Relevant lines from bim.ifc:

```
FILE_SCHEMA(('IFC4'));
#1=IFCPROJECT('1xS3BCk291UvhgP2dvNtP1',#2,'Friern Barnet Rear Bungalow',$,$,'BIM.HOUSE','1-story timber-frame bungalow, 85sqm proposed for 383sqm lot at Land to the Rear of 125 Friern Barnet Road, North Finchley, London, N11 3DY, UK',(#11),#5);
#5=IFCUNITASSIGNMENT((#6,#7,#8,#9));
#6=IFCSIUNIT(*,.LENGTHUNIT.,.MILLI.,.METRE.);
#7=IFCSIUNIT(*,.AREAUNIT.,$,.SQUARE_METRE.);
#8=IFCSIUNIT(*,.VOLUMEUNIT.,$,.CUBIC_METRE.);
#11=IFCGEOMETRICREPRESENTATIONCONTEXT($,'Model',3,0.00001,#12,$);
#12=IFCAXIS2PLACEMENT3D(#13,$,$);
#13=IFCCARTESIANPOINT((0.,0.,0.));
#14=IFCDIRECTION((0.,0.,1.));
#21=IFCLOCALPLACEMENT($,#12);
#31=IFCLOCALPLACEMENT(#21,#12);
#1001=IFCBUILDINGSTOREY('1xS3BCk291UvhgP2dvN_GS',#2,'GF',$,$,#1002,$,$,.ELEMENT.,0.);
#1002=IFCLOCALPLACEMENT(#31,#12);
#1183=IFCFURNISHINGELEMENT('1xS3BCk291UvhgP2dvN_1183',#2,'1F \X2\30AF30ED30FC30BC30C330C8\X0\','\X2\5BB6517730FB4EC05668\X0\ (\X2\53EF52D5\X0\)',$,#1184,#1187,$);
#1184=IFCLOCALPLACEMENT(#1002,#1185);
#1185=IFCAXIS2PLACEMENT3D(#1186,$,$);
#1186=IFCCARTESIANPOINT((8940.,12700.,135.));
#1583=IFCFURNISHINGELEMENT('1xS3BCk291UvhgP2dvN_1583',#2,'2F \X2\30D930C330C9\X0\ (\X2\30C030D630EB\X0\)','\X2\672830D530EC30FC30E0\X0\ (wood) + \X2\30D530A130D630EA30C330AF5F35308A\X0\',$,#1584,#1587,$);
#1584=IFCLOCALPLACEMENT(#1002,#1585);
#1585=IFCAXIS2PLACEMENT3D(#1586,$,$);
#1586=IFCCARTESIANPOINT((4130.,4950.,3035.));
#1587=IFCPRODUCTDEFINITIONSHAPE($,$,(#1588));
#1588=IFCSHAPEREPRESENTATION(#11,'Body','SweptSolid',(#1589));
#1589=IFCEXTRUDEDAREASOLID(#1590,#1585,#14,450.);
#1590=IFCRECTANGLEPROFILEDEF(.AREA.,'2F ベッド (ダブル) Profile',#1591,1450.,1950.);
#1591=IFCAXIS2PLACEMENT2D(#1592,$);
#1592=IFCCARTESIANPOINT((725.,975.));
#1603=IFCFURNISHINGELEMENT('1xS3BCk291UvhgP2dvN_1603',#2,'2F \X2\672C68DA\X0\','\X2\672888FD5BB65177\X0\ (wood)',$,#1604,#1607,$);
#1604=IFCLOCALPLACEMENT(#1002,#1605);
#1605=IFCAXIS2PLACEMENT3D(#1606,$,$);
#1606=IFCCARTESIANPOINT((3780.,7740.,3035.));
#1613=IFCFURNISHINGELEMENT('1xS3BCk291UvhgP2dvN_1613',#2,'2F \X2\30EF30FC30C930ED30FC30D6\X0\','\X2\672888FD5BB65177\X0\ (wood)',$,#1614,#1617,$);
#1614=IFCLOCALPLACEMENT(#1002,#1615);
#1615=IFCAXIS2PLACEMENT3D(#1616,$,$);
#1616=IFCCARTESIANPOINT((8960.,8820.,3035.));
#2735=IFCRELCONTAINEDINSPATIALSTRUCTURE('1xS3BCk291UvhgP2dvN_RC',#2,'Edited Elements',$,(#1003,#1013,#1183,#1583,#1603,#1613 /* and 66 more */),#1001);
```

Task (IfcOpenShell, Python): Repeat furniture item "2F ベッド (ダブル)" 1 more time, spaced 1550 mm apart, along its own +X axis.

```python
import ifcopenshell
import ifcopenshell.api.geometry
import ifcopenshell.api.root
import ifcopenshell.util.element
import ifcopenshell.util.placement
import ifcopenshell.util.unit

model = ifcopenshell.open("bim.ifc")
unit_scale = ifcopenshell.util.unit.calculate_unit_scale(model)


def reuse_history(source, copy):
    """copy_class also copies each property set's owner history, people and application; keep the originals."""
    for rel in copy.IsDefinedBy:
        if rel.is_a("IfcRelDefinesByProperties") and (history := rel.RelatingPropertyDefinition.OwnerHistory):
            rel.RelatingPropertyDefinition.OwnerHistory = source.OwnerHistory
            ifcopenshell.util.element.remove_deep2(model, history)


source = model.by_guid("1xS3BCk291UvhgP2dvN_1583")
base = ifcopenshell.util.placement.get_local_placement(source.ObjectPlacement)
step = base[:3, 0] * 1.55 / unit_scale

for i in range(1, 2):
    copy = ifcopenshell.api.root.copy_class(model, product=source)
    copy.Representation = ifcopenshell.util.element.copy_deep(
        model, source.Representation, exclude=["IfcGeometricRepresentationContext", "IfcRepresentationMap"]
    )
    reuse_history(source, copy)
    matrix = base.copy()
    matrix[:3, 3] += i * step
    print("added at", matrix[:3, 3].round(3) + 0.0)
    ifcopenshell.api.geometry.edit_object_placement(model, product=copy, matrix=matrix, is_si=False)

model.write("bim_edited.ifc")
```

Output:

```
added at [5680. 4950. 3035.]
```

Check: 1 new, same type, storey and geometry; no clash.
